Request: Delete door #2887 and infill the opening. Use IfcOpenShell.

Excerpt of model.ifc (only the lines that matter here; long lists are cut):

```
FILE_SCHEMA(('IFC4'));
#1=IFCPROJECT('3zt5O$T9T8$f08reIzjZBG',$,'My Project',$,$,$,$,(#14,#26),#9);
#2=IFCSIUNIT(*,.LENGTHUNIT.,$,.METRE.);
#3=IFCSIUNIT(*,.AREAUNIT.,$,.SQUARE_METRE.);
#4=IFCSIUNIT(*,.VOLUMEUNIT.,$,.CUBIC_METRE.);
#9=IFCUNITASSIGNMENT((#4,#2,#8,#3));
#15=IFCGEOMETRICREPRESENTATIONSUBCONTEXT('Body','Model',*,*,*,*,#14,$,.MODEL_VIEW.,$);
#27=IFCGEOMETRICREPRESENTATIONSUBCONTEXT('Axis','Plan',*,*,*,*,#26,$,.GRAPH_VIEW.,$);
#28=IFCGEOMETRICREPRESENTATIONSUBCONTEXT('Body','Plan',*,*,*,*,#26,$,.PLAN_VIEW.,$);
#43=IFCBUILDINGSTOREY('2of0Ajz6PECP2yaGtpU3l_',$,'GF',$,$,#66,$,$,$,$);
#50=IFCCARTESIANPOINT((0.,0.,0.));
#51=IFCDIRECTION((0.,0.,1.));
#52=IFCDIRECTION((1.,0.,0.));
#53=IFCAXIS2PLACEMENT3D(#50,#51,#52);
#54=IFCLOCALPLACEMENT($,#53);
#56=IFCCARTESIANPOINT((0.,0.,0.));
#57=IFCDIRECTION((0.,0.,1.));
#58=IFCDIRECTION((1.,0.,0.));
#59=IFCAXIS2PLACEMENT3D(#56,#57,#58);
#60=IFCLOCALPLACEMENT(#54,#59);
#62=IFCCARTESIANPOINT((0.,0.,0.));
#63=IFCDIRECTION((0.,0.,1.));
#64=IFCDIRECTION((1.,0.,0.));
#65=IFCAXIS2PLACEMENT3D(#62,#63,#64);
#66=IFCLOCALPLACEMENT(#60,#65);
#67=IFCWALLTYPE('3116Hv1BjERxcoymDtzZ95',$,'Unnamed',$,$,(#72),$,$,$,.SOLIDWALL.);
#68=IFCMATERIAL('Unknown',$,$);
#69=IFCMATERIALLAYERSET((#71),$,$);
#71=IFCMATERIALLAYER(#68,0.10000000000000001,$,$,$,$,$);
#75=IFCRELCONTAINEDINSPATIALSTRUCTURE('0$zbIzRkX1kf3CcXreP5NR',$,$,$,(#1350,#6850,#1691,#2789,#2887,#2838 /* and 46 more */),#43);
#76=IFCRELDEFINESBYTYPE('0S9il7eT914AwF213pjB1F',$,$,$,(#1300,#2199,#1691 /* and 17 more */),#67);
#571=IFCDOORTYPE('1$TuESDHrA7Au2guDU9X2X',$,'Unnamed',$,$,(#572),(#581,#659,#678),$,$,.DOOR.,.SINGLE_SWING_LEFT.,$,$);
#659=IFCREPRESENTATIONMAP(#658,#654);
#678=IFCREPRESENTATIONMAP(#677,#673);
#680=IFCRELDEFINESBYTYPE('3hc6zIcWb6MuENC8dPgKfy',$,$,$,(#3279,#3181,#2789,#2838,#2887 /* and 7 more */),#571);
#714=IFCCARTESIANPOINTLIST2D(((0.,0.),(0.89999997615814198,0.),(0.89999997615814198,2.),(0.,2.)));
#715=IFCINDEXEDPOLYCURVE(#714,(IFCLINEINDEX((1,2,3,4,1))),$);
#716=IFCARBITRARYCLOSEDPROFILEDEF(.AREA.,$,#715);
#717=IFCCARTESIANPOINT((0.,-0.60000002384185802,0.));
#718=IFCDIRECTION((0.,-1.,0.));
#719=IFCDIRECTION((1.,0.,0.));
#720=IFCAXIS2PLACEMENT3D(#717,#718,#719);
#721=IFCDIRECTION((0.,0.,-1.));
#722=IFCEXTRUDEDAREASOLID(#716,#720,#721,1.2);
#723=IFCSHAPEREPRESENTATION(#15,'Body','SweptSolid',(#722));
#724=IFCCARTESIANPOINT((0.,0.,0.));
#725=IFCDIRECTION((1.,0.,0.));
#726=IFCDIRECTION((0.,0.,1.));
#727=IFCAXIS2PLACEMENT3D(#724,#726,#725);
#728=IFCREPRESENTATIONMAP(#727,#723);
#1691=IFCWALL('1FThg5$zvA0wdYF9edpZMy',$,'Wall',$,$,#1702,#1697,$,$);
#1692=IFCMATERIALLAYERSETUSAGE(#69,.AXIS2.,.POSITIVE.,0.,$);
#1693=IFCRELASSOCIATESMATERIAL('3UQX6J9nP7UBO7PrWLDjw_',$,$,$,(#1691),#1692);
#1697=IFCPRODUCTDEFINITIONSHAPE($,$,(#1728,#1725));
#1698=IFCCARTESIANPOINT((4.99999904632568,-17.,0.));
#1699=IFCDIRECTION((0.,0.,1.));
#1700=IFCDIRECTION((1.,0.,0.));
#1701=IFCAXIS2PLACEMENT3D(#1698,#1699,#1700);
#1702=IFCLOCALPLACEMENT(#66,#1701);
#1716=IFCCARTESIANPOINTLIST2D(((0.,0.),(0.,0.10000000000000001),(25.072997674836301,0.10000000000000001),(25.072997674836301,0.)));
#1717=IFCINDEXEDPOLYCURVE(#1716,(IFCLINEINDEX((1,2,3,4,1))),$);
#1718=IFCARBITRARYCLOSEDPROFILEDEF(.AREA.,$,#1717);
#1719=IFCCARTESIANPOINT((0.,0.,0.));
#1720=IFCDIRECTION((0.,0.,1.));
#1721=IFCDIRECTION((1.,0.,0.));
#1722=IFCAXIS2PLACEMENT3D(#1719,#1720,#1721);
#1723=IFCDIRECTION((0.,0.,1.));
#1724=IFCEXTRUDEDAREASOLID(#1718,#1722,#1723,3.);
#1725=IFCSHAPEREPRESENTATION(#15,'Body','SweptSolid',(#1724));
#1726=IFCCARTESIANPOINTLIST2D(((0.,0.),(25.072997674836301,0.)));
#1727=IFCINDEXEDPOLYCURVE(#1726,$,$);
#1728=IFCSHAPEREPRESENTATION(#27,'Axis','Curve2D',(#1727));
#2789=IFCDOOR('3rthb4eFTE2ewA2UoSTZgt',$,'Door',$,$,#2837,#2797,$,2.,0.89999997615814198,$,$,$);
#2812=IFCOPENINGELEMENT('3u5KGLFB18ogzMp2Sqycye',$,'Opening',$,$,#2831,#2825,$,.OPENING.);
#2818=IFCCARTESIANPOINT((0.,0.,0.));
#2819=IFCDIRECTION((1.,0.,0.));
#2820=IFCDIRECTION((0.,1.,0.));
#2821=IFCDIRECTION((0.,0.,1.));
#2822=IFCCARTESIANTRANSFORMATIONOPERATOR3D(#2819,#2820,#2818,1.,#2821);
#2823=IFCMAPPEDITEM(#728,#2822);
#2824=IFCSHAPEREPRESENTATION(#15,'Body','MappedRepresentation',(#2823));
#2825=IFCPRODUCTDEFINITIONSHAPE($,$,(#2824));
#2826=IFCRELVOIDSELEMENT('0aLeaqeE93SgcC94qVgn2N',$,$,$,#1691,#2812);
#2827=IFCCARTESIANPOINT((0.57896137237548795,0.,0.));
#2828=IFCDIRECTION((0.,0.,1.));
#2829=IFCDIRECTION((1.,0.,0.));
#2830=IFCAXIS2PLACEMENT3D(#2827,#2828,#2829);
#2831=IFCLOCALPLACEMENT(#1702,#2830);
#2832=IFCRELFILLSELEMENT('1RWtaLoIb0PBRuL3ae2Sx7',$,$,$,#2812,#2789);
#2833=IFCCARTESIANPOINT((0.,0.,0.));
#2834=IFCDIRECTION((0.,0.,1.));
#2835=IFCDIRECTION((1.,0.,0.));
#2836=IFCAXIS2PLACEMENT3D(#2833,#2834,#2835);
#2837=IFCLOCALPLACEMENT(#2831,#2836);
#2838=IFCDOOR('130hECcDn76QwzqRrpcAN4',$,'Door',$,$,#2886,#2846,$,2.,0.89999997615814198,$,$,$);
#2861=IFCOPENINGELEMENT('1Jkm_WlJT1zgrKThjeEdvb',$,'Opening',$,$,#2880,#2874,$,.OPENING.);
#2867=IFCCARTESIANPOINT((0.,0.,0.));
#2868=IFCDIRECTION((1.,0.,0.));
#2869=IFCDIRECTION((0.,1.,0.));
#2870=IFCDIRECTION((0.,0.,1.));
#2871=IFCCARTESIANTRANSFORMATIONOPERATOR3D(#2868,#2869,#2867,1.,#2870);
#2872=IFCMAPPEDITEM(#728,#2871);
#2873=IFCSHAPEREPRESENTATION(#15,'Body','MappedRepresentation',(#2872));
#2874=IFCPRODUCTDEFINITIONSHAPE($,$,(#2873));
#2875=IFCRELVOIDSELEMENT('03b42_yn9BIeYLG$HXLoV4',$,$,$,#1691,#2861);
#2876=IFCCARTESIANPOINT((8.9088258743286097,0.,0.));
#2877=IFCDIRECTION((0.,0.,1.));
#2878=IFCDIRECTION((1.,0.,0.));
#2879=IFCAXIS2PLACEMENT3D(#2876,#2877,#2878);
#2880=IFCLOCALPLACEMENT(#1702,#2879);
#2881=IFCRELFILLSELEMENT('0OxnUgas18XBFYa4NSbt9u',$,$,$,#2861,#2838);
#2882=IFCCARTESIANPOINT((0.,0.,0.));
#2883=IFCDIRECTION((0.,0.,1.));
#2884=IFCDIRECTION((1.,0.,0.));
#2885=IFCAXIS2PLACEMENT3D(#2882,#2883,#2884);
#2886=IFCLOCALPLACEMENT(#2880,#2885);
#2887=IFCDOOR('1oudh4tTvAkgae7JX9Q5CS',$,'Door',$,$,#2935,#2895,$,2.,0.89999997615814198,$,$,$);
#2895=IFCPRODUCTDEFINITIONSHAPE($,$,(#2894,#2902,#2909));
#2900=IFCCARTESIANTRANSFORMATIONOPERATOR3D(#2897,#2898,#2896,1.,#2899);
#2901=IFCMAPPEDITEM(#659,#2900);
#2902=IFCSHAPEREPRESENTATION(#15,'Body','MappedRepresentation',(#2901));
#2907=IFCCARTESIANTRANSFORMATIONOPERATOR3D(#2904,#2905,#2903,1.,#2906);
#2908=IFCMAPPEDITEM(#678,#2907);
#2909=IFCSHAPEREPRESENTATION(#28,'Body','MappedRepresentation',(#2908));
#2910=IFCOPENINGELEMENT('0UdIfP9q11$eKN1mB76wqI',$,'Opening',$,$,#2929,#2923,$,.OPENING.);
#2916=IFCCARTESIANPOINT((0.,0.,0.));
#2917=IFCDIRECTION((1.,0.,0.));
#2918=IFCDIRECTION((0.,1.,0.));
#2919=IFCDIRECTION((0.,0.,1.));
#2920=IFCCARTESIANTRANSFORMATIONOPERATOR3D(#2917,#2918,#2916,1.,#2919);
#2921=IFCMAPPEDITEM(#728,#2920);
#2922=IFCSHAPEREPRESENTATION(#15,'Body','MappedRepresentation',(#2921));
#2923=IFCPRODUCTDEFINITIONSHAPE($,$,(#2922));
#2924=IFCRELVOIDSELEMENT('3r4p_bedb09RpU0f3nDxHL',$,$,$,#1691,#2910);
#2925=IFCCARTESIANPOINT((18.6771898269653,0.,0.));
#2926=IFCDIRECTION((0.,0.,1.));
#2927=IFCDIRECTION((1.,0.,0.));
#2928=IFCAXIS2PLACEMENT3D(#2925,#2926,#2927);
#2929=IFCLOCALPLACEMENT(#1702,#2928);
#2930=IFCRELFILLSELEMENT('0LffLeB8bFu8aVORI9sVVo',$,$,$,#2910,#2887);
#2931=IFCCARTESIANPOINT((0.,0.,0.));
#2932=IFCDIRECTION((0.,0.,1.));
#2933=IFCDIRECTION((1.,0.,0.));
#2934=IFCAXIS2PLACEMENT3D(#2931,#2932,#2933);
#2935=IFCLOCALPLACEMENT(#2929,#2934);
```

```python
import ifcopenshell
import ifcopenshell.api.feature
import ifcopenshell.api.root
import ifcopenshell.geom
import ifcopenshell.util.shape

model = ifcopenshell.open("model.ifc")
settings = ifcopenshell.geom.settings()


def volume(element):
    """Net volume in cubic metres, openings subtracted."""
    shape = ifcopenshell.geom.create_shape(settings, element)
    return ifcopenshell.util.shape.get_volume(shape.geometry)


door = model.by_guid("1oudh4tTvAkgae7JX9Q5CS")
opening = door.FillsVoids[0].RelatingOpeningElement
wall = opening.VoidsElements[0].RelatingBuildingElement
before = volume(wall)

ifcopenshell.api.root.remove_product(model, product=door)
ifcopenshell.api.feature.remove_feature(model, feature=opening)

after = volume(wall)

print(f"wall volume {before:.3f} -> {after:.3f} m3")

model.write("model_edited.ifc")
```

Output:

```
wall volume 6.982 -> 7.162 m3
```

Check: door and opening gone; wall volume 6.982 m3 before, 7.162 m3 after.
